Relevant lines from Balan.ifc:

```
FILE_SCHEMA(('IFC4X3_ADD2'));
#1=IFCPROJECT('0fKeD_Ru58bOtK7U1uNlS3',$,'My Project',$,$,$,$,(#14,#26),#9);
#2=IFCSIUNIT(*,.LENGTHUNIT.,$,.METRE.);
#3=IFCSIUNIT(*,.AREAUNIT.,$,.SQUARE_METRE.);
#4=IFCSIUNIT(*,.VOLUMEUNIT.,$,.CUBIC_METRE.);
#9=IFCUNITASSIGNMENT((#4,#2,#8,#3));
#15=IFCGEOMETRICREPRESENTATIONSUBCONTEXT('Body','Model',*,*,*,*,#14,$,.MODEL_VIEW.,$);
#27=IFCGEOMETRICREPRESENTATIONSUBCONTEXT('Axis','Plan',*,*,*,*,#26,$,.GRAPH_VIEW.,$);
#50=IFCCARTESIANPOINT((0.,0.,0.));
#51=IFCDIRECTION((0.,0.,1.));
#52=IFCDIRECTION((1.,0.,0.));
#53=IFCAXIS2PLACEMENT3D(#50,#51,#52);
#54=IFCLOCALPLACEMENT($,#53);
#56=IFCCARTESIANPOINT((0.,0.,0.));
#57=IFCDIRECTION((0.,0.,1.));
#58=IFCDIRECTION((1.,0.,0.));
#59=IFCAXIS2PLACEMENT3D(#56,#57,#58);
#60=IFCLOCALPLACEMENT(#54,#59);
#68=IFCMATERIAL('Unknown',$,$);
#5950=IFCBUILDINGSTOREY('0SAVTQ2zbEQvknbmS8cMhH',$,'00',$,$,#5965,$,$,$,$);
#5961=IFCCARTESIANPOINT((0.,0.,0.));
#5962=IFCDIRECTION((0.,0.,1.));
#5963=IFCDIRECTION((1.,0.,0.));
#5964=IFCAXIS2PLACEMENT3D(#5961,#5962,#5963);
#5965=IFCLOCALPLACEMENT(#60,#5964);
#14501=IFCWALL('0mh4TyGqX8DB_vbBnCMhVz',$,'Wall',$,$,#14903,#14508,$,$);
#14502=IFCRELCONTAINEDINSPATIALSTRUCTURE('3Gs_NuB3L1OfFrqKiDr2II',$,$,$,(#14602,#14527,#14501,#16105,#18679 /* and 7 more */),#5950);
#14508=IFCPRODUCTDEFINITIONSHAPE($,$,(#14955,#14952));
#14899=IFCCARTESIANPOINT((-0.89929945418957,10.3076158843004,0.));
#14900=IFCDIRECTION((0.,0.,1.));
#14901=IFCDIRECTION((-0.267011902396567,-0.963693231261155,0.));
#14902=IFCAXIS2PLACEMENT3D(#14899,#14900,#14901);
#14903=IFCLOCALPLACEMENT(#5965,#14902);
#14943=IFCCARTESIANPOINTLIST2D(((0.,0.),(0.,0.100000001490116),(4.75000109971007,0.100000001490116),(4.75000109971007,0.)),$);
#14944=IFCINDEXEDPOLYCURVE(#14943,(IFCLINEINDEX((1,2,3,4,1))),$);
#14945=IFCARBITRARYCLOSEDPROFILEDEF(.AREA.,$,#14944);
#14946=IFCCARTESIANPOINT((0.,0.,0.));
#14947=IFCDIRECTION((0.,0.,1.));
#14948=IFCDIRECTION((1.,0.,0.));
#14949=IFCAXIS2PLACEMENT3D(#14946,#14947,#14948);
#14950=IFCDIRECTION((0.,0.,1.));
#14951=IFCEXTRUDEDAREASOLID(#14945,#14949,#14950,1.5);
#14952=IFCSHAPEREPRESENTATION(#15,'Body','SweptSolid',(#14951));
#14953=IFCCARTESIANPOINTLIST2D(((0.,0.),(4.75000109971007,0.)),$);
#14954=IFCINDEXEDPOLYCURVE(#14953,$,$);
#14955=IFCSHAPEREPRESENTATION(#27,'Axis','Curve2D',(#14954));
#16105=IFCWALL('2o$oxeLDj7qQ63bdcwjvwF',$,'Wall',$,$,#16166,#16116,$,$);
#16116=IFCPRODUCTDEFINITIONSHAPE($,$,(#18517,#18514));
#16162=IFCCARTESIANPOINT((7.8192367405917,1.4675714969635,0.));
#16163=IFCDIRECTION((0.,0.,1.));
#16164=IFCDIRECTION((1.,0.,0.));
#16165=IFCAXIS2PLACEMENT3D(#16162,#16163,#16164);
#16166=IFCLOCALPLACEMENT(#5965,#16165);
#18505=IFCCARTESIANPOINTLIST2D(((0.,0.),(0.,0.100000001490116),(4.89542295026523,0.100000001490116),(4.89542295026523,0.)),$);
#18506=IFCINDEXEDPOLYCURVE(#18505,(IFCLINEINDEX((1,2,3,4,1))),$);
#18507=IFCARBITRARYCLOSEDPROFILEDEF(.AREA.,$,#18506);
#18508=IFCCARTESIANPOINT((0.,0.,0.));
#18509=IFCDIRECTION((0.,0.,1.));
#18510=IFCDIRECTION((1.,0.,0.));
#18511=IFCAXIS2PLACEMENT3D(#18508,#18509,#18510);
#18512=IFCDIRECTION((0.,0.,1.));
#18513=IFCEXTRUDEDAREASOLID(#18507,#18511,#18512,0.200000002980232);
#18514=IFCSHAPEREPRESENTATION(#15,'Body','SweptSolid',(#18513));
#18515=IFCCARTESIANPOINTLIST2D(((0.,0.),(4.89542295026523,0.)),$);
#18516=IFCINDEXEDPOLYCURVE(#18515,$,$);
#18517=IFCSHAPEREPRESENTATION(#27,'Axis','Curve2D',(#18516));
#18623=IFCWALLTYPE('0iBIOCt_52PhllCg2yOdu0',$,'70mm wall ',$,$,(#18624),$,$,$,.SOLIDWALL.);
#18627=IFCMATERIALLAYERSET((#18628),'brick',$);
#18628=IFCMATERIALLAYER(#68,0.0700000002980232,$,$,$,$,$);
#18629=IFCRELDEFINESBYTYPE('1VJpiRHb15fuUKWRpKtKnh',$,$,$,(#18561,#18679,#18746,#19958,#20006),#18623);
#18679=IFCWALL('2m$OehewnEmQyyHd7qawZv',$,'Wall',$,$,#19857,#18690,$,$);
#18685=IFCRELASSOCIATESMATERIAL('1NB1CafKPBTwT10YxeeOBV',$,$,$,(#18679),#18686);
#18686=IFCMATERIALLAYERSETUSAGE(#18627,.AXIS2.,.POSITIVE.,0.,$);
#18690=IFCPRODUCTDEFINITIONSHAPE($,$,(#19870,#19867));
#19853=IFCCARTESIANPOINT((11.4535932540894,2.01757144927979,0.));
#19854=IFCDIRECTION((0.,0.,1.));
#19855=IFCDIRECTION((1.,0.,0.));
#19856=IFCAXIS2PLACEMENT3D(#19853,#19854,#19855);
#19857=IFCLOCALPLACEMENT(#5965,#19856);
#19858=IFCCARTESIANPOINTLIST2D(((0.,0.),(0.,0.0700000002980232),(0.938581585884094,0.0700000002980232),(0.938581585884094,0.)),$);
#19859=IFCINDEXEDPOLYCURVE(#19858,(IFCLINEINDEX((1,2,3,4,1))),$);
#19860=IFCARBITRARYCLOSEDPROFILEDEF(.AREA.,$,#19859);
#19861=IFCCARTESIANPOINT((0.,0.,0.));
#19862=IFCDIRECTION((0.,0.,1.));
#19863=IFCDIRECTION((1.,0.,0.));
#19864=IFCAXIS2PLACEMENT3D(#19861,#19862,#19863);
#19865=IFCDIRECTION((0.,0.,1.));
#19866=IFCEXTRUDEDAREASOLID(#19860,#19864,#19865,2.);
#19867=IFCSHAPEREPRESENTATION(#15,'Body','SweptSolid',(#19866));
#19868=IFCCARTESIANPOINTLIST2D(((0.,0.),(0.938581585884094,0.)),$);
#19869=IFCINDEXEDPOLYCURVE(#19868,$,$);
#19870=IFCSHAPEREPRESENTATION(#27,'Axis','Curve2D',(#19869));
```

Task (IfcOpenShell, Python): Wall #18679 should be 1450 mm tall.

```python
import ifcopenshell
import ifcopenshell.geom
import ifcopenshell.util.representation
import ifcopenshell.util.shape
import ifcopenshell.util.unit

model = ifcopenshell.open("Balan.ifc")
unit_scale = ifcopenshell.util.unit.calculate_unit_scale(model)
settings = ifcopenshell.geom.settings()


def volume(element):
    """Net volume in cubic metres, openings subtracted."""
    shape = ifcopenshell.geom.create_shape(settings, element)
    return ifcopenshell.util.shape.get_volume(shape.geometry)


wall = model.by_guid("2m$OehewnEmQyyHd7qawZv")
before = volume(wall)

body = ifcopenshell.util.representation.get_representation(wall, "Model", "Body")
solid = body.Items[0]
old_height = solid.Depth
solid.Depth = 1.45 / unit_scale
after = volume(wall)

print(f"height {old_height:g} -> {solid.Depth:g}, volume {before:.3f} -> {after:.3f} m3")

model.write("Balan-out.ifc")
```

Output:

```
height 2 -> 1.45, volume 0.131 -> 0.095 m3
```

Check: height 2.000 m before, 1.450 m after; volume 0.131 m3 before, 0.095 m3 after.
